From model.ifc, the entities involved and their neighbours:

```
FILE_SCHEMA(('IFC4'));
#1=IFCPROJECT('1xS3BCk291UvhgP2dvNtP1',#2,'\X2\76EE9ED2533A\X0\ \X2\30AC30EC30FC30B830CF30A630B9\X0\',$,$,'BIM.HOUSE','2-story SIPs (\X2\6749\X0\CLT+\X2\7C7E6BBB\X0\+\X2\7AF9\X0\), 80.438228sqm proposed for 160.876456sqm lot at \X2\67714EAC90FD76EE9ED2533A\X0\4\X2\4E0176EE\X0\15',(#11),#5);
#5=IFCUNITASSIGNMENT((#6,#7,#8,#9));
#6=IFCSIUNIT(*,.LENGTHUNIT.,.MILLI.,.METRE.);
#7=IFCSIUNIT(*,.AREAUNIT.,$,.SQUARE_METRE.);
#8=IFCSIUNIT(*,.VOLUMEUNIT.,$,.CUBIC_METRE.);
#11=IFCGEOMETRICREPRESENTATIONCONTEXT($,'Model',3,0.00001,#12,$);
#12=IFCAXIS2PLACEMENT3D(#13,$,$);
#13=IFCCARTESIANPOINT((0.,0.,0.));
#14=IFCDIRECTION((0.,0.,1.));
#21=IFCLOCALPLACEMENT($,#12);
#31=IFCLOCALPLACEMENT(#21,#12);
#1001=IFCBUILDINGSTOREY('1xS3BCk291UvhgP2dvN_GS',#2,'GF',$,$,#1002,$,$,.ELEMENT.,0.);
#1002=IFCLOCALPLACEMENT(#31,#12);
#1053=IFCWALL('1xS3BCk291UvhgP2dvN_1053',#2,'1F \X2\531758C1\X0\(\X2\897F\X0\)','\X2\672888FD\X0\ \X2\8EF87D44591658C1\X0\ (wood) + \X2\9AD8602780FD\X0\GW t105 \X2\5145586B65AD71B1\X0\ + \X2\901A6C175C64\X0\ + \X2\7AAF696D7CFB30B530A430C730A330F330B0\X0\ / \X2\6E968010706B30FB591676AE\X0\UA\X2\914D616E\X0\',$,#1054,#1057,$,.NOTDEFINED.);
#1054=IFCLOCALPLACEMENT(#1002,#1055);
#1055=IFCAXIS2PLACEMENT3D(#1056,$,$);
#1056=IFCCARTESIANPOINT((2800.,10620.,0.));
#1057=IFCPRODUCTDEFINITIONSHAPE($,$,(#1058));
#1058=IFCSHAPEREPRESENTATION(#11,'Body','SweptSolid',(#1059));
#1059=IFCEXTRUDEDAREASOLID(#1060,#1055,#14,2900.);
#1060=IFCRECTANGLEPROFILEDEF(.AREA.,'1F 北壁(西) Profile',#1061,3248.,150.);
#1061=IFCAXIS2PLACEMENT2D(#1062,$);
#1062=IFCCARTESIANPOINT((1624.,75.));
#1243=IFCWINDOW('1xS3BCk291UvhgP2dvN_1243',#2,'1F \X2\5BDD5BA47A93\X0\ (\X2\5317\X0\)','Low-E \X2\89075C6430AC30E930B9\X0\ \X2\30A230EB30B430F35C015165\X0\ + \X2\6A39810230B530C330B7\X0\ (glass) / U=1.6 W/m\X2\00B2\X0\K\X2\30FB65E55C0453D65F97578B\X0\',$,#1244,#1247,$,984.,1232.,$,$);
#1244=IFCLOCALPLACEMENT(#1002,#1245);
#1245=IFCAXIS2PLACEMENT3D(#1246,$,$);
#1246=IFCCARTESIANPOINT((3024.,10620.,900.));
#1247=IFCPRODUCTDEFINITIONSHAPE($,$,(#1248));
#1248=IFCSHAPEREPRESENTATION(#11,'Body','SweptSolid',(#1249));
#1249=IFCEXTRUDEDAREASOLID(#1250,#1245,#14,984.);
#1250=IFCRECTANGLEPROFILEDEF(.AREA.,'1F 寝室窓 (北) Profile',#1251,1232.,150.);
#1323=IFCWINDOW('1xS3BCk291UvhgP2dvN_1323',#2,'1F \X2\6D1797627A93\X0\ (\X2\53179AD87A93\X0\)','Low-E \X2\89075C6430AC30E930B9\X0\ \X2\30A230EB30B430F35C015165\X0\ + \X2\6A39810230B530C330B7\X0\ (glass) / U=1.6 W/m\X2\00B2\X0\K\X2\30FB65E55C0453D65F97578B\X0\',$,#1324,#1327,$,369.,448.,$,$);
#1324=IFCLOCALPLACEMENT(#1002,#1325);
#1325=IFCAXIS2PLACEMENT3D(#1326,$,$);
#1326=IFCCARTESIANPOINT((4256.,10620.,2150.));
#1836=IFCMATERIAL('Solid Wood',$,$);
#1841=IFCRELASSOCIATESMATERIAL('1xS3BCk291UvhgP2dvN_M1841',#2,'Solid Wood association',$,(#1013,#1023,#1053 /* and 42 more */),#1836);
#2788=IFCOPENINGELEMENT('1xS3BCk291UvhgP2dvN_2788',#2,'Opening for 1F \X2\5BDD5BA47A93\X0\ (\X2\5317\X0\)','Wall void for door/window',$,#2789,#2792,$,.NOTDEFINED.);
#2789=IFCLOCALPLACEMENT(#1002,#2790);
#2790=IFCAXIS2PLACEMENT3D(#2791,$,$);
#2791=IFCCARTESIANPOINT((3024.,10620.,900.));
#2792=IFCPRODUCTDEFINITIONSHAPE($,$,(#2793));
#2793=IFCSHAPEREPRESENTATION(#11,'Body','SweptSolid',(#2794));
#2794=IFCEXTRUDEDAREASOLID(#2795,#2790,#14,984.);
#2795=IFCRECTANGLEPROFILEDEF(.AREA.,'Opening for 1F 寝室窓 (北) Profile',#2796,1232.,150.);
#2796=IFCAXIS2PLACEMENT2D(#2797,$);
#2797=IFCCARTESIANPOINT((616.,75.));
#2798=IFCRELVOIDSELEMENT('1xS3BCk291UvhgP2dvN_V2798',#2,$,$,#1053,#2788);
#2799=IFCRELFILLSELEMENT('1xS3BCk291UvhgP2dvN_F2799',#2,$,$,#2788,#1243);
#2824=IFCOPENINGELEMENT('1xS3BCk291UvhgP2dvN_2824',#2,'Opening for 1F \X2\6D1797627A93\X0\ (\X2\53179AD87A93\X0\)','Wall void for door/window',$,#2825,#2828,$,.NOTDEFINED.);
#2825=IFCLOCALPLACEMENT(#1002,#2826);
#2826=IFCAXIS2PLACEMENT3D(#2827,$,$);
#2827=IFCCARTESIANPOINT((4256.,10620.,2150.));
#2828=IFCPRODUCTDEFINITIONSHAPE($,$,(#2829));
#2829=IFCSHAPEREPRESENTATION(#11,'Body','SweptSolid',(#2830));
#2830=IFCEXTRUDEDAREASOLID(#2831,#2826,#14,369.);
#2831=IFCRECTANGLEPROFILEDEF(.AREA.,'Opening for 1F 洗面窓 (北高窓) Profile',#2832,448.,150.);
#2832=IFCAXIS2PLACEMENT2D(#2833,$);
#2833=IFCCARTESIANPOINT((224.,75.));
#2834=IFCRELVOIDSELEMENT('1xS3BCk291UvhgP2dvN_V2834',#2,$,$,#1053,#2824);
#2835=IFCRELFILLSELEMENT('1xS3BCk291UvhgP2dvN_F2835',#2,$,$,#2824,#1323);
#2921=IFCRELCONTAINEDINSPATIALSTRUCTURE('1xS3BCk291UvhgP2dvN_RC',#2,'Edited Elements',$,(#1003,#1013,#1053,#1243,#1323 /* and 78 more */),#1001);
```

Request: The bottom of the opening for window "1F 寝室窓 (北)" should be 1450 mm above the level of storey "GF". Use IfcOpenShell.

```python
import numpy as np
import ifcopenshell
import ifcopenshell.api.geometry
import ifcopenshell.geom
import ifcopenshell.util.element
import ifcopenshell.util.placement
import ifcopenshell.util.shape
import ifcopenshell.util.unit

model = ifcopenshell.open("model.ifc")
unit_scale = ifcopenshell.util.unit.calculate_unit_scale(model)

window = model.by_guid("1xS3BCk291UvhgP2dvN_1243")
opening = window.FillsVoids[0].RelatingOpeningElement
storey = ifcopenshell.util.element.get_container(window, ifc_class="IfcBuildingStorey")
level = ifcopenshell.util.placement.get_local_placement(storey.ObjectPlacement)[2, 3]

# The opening's origin need not be at the sill, so measure its lowest point.
shape = ifcopenshell.geom.create_shape(ifcopenshell.geom.settings(), opening)
bottom = ifcopenshell.util.shape.get_shape_bottom_elevation(shape, shape.geometry) / unit_scale
dz = level + 1.45 / unit_scale - bottom

shift = np.array([0.0, 0.0, dz])
# The window is not placed relative to its opening, so move both.
for product in (opening, window):
    matrix = ifcopenshell.util.placement.get_local_placement(product.ObjectPlacement)
    matrix[:3, 3] += shift
    ifcopenshell.api.geometry.edit_object_placement(model, product=product, matrix=matrix, is_si=False)

print(f"moved by {dz * unit_scale:+.3f} m")

model.write("model_updated.ifc")
```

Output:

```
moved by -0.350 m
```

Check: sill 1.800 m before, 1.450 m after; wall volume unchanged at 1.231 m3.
